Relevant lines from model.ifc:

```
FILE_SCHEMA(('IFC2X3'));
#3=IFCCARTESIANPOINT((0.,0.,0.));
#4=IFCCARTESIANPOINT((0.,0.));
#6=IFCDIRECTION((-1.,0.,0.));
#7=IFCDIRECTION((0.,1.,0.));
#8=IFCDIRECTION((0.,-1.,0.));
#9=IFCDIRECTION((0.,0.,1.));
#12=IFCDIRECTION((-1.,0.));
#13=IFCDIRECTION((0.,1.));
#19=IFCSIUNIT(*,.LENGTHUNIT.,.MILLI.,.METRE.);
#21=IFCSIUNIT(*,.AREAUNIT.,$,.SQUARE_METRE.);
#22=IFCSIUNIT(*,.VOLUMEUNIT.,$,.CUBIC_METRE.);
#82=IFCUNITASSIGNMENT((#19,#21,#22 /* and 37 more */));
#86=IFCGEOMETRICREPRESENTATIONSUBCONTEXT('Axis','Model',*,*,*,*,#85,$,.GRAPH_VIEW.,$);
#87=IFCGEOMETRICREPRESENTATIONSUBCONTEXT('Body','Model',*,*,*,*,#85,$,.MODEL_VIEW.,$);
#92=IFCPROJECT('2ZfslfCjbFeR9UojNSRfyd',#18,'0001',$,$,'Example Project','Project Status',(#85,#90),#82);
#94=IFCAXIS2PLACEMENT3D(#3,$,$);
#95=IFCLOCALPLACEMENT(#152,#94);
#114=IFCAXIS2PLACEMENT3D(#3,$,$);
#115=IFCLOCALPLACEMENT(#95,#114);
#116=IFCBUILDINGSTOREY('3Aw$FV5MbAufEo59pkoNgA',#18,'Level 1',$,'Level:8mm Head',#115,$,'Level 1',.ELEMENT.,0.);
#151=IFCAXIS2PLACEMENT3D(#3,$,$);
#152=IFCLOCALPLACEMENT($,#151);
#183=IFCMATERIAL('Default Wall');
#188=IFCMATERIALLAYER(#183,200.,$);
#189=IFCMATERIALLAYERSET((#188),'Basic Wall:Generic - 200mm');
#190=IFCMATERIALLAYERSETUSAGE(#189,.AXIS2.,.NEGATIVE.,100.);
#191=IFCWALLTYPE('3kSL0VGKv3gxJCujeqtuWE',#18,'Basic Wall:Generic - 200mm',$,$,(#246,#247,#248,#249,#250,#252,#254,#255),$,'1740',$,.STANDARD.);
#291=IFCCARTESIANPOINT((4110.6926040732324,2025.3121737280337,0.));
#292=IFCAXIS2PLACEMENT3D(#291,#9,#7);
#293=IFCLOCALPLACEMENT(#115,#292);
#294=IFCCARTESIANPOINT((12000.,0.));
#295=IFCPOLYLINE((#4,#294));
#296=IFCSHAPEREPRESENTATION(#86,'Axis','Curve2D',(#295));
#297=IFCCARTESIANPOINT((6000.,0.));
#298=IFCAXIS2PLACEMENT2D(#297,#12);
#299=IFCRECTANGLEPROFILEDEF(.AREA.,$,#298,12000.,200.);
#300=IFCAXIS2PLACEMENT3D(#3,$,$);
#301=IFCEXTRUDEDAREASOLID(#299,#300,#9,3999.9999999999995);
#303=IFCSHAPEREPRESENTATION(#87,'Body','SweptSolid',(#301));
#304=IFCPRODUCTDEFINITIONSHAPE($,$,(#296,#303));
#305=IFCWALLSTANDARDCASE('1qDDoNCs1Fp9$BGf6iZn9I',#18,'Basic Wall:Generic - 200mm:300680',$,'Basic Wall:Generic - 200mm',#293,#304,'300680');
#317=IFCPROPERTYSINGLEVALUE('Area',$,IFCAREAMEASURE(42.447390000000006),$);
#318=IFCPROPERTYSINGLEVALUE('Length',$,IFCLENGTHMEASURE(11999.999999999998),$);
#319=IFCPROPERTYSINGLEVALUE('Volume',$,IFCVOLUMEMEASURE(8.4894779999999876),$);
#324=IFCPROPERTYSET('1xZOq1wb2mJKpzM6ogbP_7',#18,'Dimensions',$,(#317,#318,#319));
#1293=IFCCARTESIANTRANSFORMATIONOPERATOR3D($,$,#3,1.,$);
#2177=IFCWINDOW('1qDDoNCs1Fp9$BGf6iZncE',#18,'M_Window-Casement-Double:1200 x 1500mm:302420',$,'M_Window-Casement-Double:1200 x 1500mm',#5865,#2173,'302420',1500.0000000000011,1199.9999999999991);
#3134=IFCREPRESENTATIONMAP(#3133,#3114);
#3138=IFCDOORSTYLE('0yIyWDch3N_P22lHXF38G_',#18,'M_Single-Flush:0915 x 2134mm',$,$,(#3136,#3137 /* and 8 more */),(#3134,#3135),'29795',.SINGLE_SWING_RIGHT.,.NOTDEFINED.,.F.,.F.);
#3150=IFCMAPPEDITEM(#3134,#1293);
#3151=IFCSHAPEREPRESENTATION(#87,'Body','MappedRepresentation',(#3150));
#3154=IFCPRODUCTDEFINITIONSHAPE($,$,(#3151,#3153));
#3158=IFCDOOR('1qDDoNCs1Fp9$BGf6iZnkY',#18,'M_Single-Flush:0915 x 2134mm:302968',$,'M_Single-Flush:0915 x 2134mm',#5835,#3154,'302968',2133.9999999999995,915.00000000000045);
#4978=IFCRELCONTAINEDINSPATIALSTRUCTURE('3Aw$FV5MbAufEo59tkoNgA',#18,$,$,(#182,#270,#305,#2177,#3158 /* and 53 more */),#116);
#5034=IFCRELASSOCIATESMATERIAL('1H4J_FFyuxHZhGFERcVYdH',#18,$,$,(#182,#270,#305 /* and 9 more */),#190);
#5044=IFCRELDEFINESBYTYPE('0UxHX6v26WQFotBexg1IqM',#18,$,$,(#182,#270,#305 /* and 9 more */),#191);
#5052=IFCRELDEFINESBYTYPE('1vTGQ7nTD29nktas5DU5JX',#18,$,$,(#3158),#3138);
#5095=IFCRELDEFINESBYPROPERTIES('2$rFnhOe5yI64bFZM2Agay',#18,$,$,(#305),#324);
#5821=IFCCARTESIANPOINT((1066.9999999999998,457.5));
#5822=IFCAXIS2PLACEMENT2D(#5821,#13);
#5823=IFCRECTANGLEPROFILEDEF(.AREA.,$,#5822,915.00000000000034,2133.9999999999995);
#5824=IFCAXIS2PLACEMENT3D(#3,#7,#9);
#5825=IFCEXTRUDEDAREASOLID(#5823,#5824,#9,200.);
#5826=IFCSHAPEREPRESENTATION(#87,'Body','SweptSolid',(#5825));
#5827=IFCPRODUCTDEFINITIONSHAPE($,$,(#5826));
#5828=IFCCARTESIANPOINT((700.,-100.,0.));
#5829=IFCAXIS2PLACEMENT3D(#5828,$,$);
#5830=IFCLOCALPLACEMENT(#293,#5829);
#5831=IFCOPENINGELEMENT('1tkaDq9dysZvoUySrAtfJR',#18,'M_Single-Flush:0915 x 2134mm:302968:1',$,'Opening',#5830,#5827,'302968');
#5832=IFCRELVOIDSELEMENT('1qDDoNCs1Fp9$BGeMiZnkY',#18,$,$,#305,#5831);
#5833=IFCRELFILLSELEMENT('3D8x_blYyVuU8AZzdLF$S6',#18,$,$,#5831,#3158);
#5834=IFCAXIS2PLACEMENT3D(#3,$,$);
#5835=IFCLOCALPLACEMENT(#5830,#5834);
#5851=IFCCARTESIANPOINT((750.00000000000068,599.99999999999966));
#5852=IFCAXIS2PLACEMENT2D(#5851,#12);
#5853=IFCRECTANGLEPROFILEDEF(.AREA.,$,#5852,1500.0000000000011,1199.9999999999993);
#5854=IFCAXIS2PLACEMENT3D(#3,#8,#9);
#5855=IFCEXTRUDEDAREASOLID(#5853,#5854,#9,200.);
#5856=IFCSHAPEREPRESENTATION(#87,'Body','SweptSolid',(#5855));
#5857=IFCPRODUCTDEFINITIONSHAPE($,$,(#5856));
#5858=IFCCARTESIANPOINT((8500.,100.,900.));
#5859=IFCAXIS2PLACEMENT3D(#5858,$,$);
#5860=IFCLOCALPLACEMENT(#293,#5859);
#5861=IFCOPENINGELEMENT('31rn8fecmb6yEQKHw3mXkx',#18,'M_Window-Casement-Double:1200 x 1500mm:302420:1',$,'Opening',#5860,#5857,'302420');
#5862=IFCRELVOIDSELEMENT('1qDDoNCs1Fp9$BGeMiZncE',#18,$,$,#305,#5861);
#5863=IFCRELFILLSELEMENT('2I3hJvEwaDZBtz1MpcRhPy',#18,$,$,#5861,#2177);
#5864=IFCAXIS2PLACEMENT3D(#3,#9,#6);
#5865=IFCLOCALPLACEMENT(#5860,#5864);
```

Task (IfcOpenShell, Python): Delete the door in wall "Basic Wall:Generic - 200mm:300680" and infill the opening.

```python
import ifcopenshell
import ifcopenshell.api.feature
import ifcopenshell.api.pset
import ifcopenshell.api.root
import ifcopenshell.geom
import ifcopenshell.util.element
import ifcopenshell.util.shape
import ifcopenshell.util.unit

model = ifcopenshell.open("model.ifc")
area_scale = ifcopenshell.util.unit.calculate_unit_scale(model, "AREAUNIT")
volume_scale = ifcopenshell.util.unit.calculate_unit_scale(model, "VOLUMEUNIT")
settings = ifcopenshell.geom.settings()


def volume(element):
    """Net volume in cubic metres, openings subtracted."""
    shape = ifcopenshell.geom.create_shape(settings, element)
    return ifcopenshell.util.shape.get_volume(shape.geometry)


door = model.by_id(3158)
opening = door.FillsVoids[0].RelatingOpeningElement
wall = opening.VoidsElements[0].RelatingBuildingElement
before = volume(wall)

ifcopenshell.api.root.remove_product(model, product=door)
ifcopenshell.api.feature.remove_feature(model, feature=opening)

after = volume(wall)
thickness = 0.2  # wall thickness in metres

# Update the wall's stored quantities.
pset = model.by_id(ifcopenshell.util.element.get_pset(wall, "Dimensions", should_inherit=False)["id"])
ifcopenshell.api.pset.edit_pset(model, pset=pset, properties={
    "Area": model.create_entity("IfcAreaMeasure", after / thickness / area_scale),
    "Volume": model.create_entity("IfcVolumeMeasure", after / volume_scale),
})

print(f"wall volume {before:.3f} -> {after:.3f} m3")

model.write("model-out.ifc")
```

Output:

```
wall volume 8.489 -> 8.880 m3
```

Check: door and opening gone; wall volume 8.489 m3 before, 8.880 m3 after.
